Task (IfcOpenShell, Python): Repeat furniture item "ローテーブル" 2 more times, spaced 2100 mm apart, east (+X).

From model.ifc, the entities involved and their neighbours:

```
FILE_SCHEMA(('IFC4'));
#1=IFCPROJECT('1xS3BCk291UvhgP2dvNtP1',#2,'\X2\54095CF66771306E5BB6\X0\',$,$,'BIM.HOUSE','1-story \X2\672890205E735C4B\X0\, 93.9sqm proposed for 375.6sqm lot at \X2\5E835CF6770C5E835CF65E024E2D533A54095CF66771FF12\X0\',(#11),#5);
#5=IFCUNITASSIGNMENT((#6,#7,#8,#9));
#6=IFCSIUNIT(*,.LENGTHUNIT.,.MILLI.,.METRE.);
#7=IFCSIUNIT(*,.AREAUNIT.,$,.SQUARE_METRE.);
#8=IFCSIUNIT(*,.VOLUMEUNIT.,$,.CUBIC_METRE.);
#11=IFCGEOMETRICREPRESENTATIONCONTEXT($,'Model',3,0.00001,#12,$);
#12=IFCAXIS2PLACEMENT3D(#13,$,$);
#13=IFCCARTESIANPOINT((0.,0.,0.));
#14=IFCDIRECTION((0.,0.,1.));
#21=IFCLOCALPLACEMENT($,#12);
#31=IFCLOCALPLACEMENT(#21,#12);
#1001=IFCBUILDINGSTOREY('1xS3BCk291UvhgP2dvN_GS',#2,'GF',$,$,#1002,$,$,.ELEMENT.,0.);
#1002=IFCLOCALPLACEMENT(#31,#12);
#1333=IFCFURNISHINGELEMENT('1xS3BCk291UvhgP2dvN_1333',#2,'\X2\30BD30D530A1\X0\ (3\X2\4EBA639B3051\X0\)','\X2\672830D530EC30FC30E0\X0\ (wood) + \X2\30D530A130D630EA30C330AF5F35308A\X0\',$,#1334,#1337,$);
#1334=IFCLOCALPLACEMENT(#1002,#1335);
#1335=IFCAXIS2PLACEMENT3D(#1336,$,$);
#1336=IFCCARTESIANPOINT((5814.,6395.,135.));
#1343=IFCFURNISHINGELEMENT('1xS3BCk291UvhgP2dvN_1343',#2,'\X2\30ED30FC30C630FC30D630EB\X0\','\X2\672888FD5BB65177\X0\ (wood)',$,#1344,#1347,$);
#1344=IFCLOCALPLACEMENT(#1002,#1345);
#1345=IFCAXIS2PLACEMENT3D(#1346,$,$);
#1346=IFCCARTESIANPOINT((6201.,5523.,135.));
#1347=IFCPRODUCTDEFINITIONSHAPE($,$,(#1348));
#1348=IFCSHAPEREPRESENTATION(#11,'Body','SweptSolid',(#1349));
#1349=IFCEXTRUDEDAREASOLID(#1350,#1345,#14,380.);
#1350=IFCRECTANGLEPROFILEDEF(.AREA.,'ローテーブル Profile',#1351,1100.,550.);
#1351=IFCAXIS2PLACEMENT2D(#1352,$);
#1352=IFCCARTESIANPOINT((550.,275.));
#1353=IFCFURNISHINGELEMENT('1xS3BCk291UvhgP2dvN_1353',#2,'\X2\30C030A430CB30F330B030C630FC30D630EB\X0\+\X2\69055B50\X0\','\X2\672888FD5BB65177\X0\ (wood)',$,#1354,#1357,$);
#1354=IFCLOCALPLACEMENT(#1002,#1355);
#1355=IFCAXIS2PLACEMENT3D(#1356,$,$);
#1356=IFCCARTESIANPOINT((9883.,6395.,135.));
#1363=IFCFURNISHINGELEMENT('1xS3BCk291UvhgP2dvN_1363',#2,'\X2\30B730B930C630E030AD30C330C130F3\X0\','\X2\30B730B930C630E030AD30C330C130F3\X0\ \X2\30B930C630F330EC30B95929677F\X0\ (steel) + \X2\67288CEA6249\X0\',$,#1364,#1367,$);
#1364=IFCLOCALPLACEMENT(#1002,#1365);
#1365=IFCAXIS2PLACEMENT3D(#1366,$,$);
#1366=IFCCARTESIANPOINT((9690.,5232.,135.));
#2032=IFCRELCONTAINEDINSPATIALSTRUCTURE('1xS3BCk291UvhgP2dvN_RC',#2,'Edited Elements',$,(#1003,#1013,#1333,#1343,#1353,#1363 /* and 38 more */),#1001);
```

```python
import numpy as np
import ifcopenshell
import ifcopenshell.api.geometry
import ifcopenshell.api.root
import ifcopenshell.util.element
import ifcopenshell.util.placement
import ifcopenshell.util.unit

model = ifcopenshell.open("model.ifc")
unit_scale = ifcopenshell.util.unit.calculate_unit_scale(model)


def reuse_history(source, copy):
    """copy_class also copies each property set's owner history, people and application; keep the originals."""
    for rel in copy.IsDefinedBy:
        if rel.is_a("IfcRelDefinesByProperties") and (history := rel.RelatingPropertyDefinition.OwnerHistory):
            rel.RelatingPropertyDefinition.OwnerHistory = source.OwnerHistory
            ifcopenshell.util.element.remove_deep2(model, history)


source = model.by_guid("1xS3BCk291UvhgP2dvN_1343")
base = ifcopenshell.util.placement.get_local_placement(source.ObjectPlacement)
step = np.array([1.0, 0.0, 0.0]) * 2.1 / unit_scale

for i in range(1, 3):
    copy = ifcopenshell.api.root.copy_class(model, product=source)
    copy.Representation = ifcopenshell.util.element.copy_deep(
        model, source.Representation, exclude=["IfcGeometricRepresentationContext", "IfcRepresentationMap"]
    )
    reuse_history(source, copy)
    matrix = base.copy()
    matrix[:3, 3] += i * step
    print("added at", matrix[:3, 3].round(3) + 0.0)
    ifcopenshell.api.geometry.edit_object_placement(model, product=copy, matrix=matrix, is_si=False)

model.write("model_edited.ifc")
```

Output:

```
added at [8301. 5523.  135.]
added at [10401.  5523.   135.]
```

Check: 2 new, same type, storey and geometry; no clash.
